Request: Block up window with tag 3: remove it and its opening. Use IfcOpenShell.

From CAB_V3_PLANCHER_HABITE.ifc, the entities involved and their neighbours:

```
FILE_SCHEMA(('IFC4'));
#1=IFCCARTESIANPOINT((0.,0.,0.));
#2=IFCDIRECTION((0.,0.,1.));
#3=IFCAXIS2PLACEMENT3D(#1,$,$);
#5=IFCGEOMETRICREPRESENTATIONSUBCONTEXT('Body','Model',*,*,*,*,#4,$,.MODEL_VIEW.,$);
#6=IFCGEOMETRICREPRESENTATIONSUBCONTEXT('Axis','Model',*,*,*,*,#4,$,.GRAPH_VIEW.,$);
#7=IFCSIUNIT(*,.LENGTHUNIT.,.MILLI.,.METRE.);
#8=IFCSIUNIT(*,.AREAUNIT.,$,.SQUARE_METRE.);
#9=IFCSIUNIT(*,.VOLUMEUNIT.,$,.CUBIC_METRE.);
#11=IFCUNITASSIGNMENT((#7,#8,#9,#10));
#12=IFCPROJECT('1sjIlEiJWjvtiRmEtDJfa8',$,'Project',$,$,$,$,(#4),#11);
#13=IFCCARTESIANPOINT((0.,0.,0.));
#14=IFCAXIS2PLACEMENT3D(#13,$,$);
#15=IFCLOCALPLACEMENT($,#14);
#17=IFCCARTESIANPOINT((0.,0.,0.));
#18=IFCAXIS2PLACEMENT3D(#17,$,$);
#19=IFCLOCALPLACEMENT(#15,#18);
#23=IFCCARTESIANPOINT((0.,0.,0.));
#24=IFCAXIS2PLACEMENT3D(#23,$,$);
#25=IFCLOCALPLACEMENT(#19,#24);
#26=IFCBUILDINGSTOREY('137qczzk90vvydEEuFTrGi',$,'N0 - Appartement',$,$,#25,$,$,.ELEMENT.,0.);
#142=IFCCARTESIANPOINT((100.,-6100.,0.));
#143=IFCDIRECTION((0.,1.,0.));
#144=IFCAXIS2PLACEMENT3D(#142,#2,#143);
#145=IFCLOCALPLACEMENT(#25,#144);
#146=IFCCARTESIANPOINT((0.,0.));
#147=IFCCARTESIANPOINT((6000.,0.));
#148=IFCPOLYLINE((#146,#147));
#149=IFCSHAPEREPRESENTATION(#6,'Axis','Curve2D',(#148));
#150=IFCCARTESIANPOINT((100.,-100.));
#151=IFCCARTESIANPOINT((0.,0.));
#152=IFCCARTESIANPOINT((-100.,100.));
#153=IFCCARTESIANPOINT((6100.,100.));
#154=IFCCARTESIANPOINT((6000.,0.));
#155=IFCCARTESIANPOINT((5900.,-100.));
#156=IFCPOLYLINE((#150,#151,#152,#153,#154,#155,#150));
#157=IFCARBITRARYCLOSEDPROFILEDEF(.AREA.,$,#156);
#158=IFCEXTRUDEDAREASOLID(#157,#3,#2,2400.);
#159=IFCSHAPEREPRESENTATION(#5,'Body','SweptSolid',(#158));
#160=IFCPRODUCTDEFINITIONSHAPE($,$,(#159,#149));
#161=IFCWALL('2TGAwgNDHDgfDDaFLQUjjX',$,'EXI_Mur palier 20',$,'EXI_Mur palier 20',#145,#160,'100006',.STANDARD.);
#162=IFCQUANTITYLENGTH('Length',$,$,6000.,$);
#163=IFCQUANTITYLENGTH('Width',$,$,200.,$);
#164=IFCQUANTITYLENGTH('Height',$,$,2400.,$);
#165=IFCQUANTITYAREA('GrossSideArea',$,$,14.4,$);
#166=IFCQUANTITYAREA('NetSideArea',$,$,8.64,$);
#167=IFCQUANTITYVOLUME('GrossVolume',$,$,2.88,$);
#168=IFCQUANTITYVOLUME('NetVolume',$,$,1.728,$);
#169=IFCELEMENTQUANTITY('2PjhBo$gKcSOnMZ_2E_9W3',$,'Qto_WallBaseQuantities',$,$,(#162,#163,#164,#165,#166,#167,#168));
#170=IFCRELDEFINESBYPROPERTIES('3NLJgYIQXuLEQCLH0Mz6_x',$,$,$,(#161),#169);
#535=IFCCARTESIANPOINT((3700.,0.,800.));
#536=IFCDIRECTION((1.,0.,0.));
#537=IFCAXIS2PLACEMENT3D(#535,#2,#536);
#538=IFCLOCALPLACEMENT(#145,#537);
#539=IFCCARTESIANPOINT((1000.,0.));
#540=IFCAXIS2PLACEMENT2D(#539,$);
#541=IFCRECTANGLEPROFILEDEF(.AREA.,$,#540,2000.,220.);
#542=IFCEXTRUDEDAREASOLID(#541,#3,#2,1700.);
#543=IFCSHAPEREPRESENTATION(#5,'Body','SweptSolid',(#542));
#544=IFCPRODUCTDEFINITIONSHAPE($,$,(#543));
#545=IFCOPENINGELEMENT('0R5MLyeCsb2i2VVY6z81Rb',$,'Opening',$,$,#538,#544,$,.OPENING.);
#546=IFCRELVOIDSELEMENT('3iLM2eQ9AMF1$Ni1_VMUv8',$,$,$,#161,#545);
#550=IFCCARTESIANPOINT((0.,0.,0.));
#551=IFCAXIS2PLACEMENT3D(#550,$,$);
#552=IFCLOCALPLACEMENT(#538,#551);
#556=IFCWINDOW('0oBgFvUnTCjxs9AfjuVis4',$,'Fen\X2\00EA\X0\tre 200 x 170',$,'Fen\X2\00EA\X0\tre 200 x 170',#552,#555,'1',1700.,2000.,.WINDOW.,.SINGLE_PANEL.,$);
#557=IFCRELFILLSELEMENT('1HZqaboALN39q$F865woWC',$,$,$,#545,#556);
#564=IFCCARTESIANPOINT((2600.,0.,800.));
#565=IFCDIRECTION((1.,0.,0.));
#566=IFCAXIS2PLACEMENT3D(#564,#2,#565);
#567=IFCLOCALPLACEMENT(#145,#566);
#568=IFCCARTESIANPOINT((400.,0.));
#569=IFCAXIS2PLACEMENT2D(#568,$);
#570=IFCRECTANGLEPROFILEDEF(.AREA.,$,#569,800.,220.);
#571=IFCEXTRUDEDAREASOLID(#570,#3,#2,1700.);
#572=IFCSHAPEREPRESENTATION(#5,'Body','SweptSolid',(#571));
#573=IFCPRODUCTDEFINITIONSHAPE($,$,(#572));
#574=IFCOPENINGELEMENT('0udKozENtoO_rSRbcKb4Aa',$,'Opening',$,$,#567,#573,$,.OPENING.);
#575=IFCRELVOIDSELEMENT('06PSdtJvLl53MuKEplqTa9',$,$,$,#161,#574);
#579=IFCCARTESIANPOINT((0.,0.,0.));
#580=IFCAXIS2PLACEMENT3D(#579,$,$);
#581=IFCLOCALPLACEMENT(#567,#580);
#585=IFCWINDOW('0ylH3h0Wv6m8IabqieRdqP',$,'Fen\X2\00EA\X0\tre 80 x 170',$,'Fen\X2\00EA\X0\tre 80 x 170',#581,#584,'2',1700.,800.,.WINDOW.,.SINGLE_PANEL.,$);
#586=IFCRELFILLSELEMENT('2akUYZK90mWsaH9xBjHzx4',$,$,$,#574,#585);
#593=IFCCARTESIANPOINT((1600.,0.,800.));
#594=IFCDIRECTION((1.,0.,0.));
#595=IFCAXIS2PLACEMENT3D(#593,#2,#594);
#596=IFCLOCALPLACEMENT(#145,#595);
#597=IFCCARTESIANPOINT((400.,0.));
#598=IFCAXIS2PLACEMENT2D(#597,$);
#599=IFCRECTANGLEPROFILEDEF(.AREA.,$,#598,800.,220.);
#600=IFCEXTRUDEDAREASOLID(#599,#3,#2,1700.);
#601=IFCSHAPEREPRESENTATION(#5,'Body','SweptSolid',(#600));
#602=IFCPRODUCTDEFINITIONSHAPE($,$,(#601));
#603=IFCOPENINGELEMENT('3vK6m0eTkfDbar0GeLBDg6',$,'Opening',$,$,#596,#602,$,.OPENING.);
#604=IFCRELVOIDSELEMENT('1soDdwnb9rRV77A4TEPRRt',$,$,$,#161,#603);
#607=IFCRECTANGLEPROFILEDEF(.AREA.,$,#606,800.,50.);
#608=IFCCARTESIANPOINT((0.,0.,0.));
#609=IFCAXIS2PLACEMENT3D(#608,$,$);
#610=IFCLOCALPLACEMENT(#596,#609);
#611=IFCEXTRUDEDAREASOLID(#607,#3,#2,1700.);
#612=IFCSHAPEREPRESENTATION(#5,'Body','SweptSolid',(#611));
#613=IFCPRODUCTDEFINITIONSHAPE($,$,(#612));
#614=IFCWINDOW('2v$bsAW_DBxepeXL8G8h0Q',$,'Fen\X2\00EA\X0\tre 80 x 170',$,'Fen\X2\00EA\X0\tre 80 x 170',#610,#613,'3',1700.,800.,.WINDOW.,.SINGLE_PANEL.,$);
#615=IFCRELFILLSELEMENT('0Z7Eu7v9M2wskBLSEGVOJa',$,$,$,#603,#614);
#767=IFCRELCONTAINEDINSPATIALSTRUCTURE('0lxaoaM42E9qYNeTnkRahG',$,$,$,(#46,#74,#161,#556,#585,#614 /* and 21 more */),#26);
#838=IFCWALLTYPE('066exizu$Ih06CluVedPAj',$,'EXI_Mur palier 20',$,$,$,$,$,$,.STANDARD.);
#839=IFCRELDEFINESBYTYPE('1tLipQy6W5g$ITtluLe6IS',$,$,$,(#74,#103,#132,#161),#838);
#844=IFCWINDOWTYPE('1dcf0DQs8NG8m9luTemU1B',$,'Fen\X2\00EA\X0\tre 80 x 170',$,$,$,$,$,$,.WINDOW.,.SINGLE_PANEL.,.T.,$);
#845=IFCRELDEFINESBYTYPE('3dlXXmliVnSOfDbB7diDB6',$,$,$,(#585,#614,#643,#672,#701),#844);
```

```python
import ifcopenshell
import ifcopenshell.api.feature
import ifcopenshell.api.pset
import ifcopenshell.api.root
import ifcopenshell.geom
import ifcopenshell.util.element
import ifcopenshell.util.shape
import ifcopenshell.util.unit

model = ifcopenshell.open("CAB_V3_PLANCHER_HABITE.ifc")
area_scale = ifcopenshell.util.unit.calculate_unit_scale(model, "AREAUNIT")
volume_scale = ifcopenshell.util.unit.calculate_unit_scale(model, "VOLUMEUNIT")
settings = ifcopenshell.geom.settings()


def volume(element):
    """Net volume in cubic metres, openings subtracted."""
    shape = ifcopenshell.geom.create_shape(settings, element)
    return ifcopenshell.util.shape.get_volume(shape.geometry)


window = model.by_id(614)
opening = window.FillsVoids[0].RelatingOpeningElement
wall = opening.VoidsElements[0].RelatingBuildingElement
before = volume(wall)

ifcopenshell.api.root.remove_product(model, product=window)
ifcopenshell.api.feature.remove_feature(model, feature=opening)

after = volume(wall)
thickness = 0.2  # wall thickness in metres

# Update the wall's stored quantities.
qto = model.by_id(ifcopenshell.util.element.get_pset(wall, "Qto_WallBaseQuantities", should_inherit=False)["id"])
ifcopenshell.api.pset.edit_qto(model, qto=qto, properties={
    "NetSideArea": after / thickness / area_scale,
    "NetVolume": after / volume_scale,
})

print(f"wall volume {before:.3f} -> {after:.3f} m3")

model.write("CAB_V3_PLANCHER_HABITE_rev.ifc")
```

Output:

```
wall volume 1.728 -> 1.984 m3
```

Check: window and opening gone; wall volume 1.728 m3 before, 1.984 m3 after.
